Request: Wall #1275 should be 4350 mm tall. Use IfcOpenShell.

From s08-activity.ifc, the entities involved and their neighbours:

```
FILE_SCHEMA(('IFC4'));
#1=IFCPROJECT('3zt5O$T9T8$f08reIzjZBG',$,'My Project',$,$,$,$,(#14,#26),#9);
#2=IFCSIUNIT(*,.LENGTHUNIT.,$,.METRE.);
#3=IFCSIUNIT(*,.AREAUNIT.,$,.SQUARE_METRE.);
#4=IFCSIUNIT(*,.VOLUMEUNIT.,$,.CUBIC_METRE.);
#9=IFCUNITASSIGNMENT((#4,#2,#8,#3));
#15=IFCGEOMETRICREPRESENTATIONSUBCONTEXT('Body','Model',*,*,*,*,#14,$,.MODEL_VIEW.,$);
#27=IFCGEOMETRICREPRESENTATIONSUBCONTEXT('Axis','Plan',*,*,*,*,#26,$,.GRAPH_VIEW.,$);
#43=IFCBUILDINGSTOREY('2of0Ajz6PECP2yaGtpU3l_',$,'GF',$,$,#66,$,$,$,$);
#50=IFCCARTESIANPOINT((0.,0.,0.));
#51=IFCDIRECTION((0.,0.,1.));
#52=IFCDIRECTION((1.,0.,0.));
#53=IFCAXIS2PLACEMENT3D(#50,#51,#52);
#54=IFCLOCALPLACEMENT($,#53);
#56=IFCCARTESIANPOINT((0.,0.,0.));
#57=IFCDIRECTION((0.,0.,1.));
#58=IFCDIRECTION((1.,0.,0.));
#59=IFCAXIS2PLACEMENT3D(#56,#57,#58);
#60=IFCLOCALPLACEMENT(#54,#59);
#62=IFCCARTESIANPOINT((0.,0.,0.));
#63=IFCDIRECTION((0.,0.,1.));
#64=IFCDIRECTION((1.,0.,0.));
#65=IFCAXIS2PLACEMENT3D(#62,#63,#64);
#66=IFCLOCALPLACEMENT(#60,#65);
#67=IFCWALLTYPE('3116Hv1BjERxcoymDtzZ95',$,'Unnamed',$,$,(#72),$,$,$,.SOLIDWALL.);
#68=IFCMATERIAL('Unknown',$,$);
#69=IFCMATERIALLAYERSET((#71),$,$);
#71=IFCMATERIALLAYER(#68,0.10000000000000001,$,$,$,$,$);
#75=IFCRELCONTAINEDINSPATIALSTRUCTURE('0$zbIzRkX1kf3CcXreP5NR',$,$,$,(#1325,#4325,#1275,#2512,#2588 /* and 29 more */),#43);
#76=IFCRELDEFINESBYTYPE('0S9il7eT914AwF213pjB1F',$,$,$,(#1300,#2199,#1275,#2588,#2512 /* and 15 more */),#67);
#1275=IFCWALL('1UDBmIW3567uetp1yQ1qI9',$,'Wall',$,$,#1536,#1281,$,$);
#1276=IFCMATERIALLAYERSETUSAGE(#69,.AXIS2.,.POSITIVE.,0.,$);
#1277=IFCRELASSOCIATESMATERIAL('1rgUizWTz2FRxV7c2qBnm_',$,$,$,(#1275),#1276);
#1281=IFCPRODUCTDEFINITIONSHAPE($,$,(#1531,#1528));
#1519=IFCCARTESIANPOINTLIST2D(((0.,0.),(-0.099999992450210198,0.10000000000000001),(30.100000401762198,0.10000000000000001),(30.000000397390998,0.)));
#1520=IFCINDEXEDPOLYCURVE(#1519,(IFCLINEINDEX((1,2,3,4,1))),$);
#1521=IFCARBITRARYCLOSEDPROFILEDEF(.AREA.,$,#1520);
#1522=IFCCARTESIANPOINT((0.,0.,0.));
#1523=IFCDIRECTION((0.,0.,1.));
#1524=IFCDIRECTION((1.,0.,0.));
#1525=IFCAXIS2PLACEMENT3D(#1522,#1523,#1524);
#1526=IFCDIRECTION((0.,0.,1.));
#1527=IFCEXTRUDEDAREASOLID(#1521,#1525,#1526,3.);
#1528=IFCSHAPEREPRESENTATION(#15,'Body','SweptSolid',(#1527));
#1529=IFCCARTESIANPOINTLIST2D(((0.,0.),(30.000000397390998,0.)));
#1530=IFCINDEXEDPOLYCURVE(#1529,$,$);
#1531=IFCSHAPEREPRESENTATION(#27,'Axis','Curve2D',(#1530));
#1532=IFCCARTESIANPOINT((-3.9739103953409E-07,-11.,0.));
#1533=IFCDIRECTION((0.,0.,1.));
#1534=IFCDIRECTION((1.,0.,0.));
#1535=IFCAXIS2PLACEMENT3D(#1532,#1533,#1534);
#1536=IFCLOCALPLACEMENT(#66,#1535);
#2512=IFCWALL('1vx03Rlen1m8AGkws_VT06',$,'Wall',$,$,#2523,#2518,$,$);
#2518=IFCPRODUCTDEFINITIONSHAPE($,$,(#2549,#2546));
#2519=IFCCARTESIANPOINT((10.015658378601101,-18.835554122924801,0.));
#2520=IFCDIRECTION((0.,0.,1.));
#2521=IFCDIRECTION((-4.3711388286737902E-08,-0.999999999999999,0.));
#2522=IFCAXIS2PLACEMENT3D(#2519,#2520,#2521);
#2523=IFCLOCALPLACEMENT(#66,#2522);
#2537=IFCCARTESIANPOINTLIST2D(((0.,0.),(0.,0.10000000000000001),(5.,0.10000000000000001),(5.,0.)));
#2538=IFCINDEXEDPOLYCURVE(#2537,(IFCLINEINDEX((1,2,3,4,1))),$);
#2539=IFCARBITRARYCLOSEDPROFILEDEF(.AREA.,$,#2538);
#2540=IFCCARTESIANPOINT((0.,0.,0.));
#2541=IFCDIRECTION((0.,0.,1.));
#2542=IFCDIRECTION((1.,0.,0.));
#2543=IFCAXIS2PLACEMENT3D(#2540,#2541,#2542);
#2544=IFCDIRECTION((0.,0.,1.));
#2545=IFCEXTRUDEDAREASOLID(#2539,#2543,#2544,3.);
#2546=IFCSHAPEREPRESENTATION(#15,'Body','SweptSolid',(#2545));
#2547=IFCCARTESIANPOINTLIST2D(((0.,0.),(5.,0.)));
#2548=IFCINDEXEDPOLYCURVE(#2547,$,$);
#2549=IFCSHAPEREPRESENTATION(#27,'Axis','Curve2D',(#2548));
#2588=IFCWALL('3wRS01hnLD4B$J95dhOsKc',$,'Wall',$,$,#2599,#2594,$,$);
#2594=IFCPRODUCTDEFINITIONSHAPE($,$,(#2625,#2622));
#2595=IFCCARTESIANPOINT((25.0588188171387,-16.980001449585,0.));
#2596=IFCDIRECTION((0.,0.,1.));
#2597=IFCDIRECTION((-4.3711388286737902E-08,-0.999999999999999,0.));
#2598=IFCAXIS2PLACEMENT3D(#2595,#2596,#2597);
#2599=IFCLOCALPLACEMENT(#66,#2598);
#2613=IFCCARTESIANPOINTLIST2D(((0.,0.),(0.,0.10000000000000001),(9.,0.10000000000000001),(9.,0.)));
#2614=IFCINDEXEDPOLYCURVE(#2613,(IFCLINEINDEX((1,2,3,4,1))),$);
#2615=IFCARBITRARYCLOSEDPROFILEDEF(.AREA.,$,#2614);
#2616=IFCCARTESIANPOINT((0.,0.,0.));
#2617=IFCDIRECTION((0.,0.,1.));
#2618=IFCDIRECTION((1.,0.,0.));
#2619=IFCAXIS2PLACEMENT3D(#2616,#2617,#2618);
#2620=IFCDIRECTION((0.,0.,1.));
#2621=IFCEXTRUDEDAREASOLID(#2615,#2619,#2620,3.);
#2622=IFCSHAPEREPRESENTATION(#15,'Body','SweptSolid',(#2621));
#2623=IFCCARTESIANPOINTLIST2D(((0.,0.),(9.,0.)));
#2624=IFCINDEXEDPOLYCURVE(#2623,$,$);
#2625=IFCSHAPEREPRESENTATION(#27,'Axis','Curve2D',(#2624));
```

```python
import ifcopenshell
import ifcopenshell.geom
import ifcopenshell.util.representation
import ifcopenshell.util.shape
import ifcopenshell.util.unit

model = ifcopenshell.open("s08-activity.ifc")
unit_scale = ifcopenshell.util.unit.calculate_unit_scale(model)
settings = ifcopenshell.geom.settings()


def volume(element):
    """Net volume in cubic metres, openings subtracted."""
    shape = ifcopenshell.geom.create_shape(settings, element)
    return ifcopenshell.util.shape.get_volume(shape.geometry)


wall = model.by_guid("1UDBmIW3567uetp1yQ1qI9")
before = volume(wall)

body = ifcopenshell.util.representation.get_representation(wall, "Model", "Body")
solid = body.Items[0]
old_height = solid.Depth
solid.Depth = 4.35 / unit_scale
after = volume(wall)

print(f"height {old_height:g} -> {solid.Depth:g}, volume {before:.3f} -> {after:.3f} m3")

model.write("s08-activity-out.ifc")
```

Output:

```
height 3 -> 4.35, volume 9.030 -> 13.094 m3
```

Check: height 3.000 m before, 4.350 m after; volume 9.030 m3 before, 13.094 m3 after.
